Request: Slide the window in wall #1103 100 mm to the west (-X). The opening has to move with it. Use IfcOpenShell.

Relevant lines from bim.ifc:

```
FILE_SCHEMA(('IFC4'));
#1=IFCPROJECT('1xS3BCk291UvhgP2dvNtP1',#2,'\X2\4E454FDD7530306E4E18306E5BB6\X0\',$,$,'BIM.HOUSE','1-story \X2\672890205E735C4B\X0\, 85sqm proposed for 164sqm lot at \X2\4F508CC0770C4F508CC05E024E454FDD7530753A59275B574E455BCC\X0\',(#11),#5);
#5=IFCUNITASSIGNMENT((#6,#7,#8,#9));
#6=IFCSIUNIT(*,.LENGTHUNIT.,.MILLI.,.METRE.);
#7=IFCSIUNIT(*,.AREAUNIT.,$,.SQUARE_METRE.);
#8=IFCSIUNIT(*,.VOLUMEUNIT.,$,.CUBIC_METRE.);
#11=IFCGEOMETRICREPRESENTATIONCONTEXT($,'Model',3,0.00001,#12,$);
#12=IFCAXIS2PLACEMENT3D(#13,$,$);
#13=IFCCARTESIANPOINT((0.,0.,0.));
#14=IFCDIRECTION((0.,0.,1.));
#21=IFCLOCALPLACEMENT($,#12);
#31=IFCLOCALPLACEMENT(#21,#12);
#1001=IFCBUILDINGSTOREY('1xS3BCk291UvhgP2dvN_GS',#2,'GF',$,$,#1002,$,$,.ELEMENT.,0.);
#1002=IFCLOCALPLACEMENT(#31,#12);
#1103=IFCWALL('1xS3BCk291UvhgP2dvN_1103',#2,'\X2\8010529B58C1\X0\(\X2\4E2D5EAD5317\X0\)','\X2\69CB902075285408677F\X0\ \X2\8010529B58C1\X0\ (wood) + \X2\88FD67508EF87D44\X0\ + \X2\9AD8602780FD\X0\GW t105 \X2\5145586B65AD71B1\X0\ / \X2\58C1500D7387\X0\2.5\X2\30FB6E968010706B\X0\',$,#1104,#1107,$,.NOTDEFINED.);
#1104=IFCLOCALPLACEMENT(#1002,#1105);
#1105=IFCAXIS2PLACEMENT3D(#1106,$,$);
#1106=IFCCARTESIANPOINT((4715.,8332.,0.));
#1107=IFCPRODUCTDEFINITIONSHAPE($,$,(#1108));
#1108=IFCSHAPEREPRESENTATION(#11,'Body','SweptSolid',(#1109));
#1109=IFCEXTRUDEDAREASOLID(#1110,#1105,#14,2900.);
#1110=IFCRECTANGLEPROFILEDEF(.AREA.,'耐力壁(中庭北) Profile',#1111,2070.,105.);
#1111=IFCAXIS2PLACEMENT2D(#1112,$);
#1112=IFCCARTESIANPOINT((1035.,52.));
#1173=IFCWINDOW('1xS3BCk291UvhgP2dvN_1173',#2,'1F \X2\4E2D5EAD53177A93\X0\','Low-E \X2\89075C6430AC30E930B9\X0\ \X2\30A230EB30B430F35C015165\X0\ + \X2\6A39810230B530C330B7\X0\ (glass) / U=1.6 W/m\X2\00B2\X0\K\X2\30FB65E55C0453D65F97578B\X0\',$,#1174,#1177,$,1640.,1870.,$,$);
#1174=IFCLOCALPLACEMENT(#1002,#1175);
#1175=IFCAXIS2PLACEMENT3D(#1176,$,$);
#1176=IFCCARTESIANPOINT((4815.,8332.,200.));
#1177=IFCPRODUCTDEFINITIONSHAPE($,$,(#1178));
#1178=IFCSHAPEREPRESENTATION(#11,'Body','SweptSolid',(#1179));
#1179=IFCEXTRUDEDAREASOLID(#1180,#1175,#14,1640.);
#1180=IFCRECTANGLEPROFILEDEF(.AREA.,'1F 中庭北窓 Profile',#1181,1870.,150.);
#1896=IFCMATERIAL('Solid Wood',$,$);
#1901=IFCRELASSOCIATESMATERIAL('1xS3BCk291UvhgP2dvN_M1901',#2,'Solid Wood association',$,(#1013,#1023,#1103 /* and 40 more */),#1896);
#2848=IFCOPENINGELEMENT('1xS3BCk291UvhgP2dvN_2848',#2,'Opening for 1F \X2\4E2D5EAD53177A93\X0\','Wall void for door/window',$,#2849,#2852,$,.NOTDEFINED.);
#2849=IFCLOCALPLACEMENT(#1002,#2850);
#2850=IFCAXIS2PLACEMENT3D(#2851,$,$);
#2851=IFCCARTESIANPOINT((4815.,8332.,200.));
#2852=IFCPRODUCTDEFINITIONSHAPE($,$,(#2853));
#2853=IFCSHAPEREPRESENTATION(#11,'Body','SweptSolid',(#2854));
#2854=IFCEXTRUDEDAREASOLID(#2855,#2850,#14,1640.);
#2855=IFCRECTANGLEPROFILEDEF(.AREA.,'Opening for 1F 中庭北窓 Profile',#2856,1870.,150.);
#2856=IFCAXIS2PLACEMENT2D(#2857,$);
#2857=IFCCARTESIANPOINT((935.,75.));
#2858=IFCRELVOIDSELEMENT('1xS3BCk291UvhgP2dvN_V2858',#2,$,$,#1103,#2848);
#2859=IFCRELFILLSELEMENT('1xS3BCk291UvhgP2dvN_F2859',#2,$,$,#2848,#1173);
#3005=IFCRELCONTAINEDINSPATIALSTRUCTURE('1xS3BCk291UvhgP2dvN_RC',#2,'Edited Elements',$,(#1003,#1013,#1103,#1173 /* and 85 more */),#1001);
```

```python
import ifcopenshell
import ifcopenshell.api.geometry
import ifcopenshell.util.placement

model = ifcopenshell.open("bim.ifc")

window = model.by_guid("1xS3BCk291UvhgP2dvN_1173")
opening = window.FillsVoids[0].RelatingOpeningElement
wall = opening.VoidsElements[0].RelatingBuildingElement

wall_matrix = ifcopenshell.util.placement.get_local_placement(wall.ObjectPlacement)
shift = wall_matrix[:3, 0] * -100.0
before = ifcopenshell.util.placement.get_local_placement(window.ObjectPlacement)[:3, 3].copy()

# The window is not placed relative to its opening, so move both.
for product in (opening, window):
    matrix = ifcopenshell.util.placement.get_local_placement(product.ObjectPlacement)
    matrix[:3, 3] += shift
    ifcopenshell.api.geometry.edit_object_placement(model, product=product, matrix=matrix, is_si=False)

after = ifcopenshell.util.placement.get_local_placement(window.ObjectPlacement)[:3, 3]
print("window moved by", (after - before).round(3) + 0.0)

model.write("bim_edited.ifc")
```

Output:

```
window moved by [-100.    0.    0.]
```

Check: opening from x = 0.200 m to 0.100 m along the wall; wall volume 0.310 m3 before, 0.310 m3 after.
